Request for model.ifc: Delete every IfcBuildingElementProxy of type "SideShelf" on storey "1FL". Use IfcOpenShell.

First a look at what the model holds.

```python
import ifcopenshell
import ifcopenshell.util.element

model = ifcopenshell.open("model.ifc")
print(model.schema)
storey = next(s for s in model.by_type("IfcBuildingStorey") if s.Name == "1FL")
proxies = [e for e in ifcopenshell.util.element.get_decomposition(storey) if e.is_a("IfcBuildingElementProxy")]
seen = {}
for e in proxies:
    element_type = ifcopenshell.util.element.get_type(e)
    name = element_type.Name if element_type not in (None, e) else None
    seen[name] = seen.get(name, 0) + 1
for name, count in sorted(seen.items(), key=str):
    print(count, "x", name)
```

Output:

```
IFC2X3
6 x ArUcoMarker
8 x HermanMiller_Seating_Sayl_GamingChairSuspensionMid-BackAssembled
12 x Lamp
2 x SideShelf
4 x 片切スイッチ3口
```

```python
import ifcopenshell
import ifcopenshell.api.root
import ifcopenshell.util.element

model = ifcopenshell.open("model.ifc")

storey = next(s for s in model.by_type("IfcBuildingStorey") if s.Name == "1FL")
proxies = [e for e in ifcopenshell.util.element.get_decomposition(storey) if e.is_a("IfcBuildingElementProxy")]
targets = [e for e in proxies if (t := ifcopenshell.util.element.get_type(e)) not in (None, e) and t.Name == "SideShelf"]

for e in targets:
    ifcopenshell.api.root.remove_product(model, product=e)
print(len(targets), "removed")

model.write("model_v2.ifc")
```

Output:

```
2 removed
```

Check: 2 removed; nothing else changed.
